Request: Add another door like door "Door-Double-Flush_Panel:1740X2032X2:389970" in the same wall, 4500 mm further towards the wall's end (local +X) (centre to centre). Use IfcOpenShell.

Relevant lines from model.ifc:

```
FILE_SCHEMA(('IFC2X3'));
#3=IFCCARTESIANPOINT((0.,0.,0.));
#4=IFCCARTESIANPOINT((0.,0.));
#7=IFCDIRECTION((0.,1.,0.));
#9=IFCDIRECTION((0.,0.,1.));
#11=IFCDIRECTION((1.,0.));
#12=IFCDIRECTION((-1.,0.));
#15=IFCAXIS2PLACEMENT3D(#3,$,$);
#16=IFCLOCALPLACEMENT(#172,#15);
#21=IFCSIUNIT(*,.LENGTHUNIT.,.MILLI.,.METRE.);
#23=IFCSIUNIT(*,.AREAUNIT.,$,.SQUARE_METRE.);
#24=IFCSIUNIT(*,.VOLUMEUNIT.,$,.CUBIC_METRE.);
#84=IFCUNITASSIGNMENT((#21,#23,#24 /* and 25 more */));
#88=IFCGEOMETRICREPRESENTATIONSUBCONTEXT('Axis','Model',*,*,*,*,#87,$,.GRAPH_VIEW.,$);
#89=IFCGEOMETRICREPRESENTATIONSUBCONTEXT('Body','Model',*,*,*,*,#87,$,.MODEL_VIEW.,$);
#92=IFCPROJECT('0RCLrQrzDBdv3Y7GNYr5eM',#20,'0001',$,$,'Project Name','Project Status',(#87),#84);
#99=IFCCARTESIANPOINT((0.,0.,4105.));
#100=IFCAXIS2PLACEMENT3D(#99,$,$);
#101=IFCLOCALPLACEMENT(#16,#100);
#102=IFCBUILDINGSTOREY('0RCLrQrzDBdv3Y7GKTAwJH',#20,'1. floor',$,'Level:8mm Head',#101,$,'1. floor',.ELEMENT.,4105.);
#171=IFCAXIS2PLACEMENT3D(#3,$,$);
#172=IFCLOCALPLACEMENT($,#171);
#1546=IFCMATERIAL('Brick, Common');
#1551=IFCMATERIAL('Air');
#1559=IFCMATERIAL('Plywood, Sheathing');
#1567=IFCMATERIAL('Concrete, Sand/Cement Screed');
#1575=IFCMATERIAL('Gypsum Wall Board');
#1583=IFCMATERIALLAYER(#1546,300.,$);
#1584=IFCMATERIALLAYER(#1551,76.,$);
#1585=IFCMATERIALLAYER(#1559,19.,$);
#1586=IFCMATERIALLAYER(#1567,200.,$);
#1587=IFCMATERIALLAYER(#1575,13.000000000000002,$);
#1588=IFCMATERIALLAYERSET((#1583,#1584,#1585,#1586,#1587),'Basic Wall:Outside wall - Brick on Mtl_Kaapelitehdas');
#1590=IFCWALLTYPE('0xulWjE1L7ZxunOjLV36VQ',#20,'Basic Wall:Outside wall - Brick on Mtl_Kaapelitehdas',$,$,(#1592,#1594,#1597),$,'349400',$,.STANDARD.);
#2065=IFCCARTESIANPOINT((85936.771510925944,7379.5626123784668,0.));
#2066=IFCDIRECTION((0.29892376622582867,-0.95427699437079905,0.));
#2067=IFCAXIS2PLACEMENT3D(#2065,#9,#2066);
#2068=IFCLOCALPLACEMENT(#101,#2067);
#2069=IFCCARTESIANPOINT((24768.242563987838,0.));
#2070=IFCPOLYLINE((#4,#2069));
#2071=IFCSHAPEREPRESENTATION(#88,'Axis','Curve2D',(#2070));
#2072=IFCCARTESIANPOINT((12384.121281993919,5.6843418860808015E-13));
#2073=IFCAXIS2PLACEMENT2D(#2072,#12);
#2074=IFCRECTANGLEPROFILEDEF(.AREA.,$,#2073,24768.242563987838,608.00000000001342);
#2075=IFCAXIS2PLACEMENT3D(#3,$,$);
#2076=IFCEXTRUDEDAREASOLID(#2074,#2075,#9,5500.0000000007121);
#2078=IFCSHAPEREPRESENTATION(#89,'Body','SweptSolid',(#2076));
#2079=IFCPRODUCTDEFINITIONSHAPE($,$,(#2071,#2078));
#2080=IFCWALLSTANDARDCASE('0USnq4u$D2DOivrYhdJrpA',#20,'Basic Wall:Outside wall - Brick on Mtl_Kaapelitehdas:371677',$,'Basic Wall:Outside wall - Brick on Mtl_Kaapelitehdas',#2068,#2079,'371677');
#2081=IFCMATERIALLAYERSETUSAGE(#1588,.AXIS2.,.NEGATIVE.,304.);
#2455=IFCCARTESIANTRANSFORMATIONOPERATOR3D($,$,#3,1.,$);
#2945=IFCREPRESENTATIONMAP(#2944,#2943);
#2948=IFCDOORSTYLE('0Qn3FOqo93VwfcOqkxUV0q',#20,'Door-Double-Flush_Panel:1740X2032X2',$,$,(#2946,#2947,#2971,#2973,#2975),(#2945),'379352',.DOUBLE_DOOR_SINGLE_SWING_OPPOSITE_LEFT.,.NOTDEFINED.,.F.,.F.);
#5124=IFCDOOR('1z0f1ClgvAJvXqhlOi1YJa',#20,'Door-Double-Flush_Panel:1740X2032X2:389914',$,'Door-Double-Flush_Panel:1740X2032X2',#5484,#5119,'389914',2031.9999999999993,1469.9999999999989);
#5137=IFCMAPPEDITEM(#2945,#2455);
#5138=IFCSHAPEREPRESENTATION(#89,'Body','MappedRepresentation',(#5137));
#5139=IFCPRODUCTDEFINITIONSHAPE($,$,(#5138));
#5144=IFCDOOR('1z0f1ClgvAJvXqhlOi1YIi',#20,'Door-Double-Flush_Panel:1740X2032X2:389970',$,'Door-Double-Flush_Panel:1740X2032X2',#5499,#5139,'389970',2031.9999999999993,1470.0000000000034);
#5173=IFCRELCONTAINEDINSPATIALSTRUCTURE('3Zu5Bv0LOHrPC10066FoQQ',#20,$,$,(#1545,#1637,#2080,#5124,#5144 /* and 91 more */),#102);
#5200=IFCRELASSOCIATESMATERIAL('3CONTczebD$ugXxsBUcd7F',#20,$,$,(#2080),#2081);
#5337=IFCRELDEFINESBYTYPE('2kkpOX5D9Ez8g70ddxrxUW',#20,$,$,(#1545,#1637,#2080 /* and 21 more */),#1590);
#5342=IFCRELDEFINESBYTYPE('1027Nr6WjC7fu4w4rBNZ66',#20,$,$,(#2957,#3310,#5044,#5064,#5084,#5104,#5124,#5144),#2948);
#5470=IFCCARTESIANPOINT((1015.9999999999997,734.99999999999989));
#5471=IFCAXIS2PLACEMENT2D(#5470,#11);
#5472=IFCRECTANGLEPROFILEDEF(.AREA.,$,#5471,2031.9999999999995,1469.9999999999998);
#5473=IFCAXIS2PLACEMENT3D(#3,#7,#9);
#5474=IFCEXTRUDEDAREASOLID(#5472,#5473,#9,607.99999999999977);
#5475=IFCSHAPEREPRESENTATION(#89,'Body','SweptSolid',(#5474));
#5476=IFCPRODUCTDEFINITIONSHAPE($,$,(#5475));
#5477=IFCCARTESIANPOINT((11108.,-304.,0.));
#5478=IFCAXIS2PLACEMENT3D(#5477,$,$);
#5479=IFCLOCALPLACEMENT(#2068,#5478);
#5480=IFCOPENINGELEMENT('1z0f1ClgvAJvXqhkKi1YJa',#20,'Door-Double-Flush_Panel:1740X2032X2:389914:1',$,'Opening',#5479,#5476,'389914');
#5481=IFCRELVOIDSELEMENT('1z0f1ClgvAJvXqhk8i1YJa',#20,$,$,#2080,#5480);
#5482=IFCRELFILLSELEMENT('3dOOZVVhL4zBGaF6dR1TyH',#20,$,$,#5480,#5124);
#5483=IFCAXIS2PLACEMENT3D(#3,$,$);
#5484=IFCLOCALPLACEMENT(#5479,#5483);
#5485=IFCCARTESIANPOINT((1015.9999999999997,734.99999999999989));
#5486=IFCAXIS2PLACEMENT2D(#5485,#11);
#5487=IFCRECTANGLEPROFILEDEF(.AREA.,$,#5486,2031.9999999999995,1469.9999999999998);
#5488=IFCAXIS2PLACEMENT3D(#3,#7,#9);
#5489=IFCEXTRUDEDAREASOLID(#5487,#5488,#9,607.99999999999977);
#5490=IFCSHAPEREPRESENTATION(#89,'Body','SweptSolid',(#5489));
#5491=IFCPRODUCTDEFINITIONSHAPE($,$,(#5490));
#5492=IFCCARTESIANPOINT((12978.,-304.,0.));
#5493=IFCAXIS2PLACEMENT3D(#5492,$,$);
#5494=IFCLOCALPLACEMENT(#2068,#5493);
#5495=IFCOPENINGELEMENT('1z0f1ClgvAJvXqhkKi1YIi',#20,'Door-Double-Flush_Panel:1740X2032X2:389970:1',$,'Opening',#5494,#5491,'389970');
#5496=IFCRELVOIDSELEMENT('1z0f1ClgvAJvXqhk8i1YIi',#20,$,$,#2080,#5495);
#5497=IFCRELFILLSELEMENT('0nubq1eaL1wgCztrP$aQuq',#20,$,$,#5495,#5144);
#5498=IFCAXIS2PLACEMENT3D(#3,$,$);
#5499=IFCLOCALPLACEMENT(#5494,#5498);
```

```python
import ifcopenshell
import ifcopenshell.api.feature
import ifcopenshell.api.geometry
import ifcopenshell.api.root
import ifcopenshell.geom
import ifcopenshell.util.element
import ifcopenshell.util.placement
import ifcopenshell.util.shape
import ifcopenshell.util.unit

model = ifcopenshell.open("model.ifc")
unit_scale = ifcopenshell.util.unit.calculate_unit_scale(model)
settings = ifcopenshell.geom.settings()


def volume(element):
    """Net volume in cubic metres, openings subtracted."""
    shape = ifcopenshell.geom.create_shape(settings, element)
    return ifcopenshell.util.shape.get_volume(shape.geometry)


def reuse_history(source, copy):
    """copy_class also copies each property set's owner history, people and application; keep the originals."""
    for rel in copy.IsDefinedBy:
        if rel.is_a("IfcRelDefinesByProperties") and (history := rel.RelatingPropertyDefinition.OwnerHistory):
            rel.RelatingPropertyDefinition.OwnerHistory = source.OwnerHistory
            ifcopenshell.util.element.remove_deep2(model, history)


door = model.by_guid("1z0f1ClgvAJvXqhlOi1YIi")
opening = door.FillsVoids[0].RelatingOpeningElement
wall = opening.VoidsElements[0].RelatingBuildingElement
before = volume(wall)
shift = ifcopenshell.util.placement.get_local_placement(wall.ObjectPlacement)[:3, 0] * 4.5 / unit_scale

# copy_class copies the void relationship, type, container and properties, but no geometry.
new_opening = ifcopenshell.api.root.copy_class(model, product=opening)
new_opening.Representation = ifcopenshell.util.element.copy_deep(
    model, opening.Representation, exclude=["IfcGeometricRepresentationContext", "IfcRepresentationMap"]
)
new_opening.Name = "Door-Double-Flush_Panel:1740X2032X2"
new_opening.Tag = None
new_door = ifcopenshell.api.root.copy_class(model, product=door)
new_door.Representation = ifcopenshell.util.element.copy_deep(
    model, door.Representation, exclude=["IfcGeometricRepresentationContext", "IfcRepresentationMap"]
)
new_door.Name = "Door-Double-Flush_Panel:1740X2032X2"
new_door.Tag = None
reuse_history(door, new_door)
fills = ifcopenshell.api.feature.add_filling(model, opening=new_opening, element=new_door)
fills.OwnerHistory = new_door.OwnerHistory  # required in IFC2X3

for old, new in ((opening, new_opening), (door, new_door)):
    matrix = ifcopenshell.util.placement.get_local_placement(old.ObjectPlacement)
    matrix[:3, 3] += shift
    ifcopenshell.api.geometry.edit_object_placement(model, product=new, matrix=matrix, is_si=False)

after = volume(wall)

print(f"wall volume {before:.3f} -> {after:.3f} m3")

model.write("model_v2.ifc")
```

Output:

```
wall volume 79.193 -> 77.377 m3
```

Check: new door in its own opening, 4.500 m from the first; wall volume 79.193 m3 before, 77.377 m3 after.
